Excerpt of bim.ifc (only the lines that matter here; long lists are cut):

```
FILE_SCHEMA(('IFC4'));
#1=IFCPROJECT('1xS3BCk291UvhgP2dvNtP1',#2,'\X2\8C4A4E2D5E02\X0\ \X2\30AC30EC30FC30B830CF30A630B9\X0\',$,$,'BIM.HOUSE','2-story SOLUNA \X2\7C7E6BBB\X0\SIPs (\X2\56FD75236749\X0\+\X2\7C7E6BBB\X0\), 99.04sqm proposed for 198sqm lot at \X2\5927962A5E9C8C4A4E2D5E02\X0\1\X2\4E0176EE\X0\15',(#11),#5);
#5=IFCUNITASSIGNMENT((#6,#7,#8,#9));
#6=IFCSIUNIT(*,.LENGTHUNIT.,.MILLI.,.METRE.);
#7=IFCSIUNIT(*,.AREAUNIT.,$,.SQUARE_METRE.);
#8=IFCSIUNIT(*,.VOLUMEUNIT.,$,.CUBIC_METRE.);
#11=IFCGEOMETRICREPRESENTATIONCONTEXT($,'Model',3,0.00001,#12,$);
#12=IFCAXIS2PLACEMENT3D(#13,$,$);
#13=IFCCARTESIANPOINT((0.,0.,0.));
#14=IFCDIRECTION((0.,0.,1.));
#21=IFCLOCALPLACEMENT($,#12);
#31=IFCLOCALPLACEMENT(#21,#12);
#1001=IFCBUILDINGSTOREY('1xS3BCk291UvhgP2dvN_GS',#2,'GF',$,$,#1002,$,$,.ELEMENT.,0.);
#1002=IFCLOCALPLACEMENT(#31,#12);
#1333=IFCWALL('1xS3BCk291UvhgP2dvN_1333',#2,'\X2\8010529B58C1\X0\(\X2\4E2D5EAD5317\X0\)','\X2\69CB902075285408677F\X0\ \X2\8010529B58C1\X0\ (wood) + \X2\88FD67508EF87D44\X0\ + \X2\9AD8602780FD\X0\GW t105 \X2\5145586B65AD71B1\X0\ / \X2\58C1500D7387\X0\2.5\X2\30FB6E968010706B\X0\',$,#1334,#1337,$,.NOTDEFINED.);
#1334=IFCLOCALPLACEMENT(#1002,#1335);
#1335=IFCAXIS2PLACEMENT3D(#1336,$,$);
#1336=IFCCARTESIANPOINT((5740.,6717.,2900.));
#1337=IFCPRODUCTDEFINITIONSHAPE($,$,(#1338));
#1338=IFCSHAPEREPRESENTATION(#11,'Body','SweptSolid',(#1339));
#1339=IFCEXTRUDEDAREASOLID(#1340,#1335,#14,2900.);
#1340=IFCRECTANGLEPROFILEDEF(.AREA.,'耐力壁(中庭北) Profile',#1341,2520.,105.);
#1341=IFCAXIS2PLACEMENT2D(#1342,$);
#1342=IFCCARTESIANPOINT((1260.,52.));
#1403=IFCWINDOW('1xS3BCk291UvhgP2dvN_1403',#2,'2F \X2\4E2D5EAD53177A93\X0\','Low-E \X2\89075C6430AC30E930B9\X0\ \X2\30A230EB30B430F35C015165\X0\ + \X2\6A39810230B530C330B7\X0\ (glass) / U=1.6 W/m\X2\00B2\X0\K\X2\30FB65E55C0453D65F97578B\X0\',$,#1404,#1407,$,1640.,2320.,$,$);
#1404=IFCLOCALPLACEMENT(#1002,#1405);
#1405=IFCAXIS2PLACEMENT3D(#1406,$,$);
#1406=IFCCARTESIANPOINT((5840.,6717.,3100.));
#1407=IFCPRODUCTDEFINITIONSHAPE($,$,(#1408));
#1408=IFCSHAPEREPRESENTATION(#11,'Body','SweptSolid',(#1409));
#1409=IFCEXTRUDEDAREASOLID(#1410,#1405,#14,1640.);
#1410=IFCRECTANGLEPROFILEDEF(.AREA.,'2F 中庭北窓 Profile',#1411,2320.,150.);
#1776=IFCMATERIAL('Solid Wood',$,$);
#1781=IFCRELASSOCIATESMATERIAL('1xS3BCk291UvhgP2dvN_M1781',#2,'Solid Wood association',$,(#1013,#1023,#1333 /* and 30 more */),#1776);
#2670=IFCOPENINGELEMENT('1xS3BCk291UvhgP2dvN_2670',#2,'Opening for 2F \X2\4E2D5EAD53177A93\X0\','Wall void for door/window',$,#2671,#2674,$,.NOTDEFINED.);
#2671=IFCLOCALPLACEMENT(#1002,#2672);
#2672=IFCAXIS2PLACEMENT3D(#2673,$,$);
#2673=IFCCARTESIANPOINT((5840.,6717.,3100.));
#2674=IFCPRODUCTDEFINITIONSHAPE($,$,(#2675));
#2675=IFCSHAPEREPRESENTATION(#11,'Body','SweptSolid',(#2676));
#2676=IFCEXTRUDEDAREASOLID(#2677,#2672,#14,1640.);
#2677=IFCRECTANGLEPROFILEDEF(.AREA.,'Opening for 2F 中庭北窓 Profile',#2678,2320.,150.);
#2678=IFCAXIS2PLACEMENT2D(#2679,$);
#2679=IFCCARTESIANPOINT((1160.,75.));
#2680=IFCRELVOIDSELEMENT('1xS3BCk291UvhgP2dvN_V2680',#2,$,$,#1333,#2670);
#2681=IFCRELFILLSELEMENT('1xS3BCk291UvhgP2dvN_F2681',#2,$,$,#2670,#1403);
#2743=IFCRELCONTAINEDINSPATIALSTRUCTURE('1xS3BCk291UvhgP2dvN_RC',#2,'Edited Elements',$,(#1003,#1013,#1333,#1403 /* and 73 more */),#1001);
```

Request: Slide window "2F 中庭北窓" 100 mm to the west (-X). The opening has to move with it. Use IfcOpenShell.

```python
import ifcopenshell
import ifcopenshell.api.geometry
import ifcopenshell.util.placement

model = ifcopenshell.open("bim.ifc")

window = model.by_id(1403)
opening = window.FillsVoids[0].RelatingOpeningElement
wall = opening.VoidsElements[0].RelatingBuildingElement

wall_matrix = ifcopenshell.util.placement.get_local_placement(wall.ObjectPlacement)
shift = wall_matrix[:3, 0] * -100.0
before = ifcopenshell.util.placement.get_local_placement(window.ObjectPlacement)[:3, 3].copy()

# The window is not placed relative to its opening, so move both.
for product in (opening, window):
    matrix = ifcopenshell.util.placement.get_local_placement(product.ObjectPlacement)
    matrix[:3, 3] += shift
    ifcopenshell.api.geometry.edit_object_placement(model, product=product, matrix=matrix, is_si=False)

after = ifcopenshell.util.placement.get_local_placement(window.ObjectPlacement)[:3, 3]
print("window moved by", (after - before).round(3) + 0.0)

model.write("bim_v2.ifc")
```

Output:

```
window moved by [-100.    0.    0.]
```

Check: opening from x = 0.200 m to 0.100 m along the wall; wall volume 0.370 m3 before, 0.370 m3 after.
